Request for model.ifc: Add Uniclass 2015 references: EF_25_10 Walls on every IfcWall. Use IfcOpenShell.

First a look at what the model holds.

```python
import ifcopenshell

model = ifcopenshell.open("model.ifc")
print(model.schema)
print("classifications:", [c.Name for c in model.by_type("IfcClassification")])
for ifc_class in ("IfcDoor", "IfcRoof", "IfcStair", "IfcWall", "IfcWindow"):
    print(ifc_class, len(model.by_type(ifc_class)))
```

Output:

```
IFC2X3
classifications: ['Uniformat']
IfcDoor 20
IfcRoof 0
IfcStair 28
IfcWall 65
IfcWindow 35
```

```python
import ifcopenshell
import ifcopenshell.api.classification

model = ifcopenshell.open("model.ifc")

# IFC2X3 requires Source and Edition and has no link from the project to the system.
system = model.create_entity("IfcClassification", Source="NBS", Edition="2015", Name="Uniclass 2015")

codes = {
    "IfcWall": ("EF_25_10", "Walls"),
}
for ifc_class, (code, name) in codes.items():
    products = model.by_type(ifc_class)
    ifcopenshell.api.classification.add_reference(
        model, products=products, classification=system, identification=code, name=name
    )
    print(code, len(products))

model.write("model_rev.ifc")
```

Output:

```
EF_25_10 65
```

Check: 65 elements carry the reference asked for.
